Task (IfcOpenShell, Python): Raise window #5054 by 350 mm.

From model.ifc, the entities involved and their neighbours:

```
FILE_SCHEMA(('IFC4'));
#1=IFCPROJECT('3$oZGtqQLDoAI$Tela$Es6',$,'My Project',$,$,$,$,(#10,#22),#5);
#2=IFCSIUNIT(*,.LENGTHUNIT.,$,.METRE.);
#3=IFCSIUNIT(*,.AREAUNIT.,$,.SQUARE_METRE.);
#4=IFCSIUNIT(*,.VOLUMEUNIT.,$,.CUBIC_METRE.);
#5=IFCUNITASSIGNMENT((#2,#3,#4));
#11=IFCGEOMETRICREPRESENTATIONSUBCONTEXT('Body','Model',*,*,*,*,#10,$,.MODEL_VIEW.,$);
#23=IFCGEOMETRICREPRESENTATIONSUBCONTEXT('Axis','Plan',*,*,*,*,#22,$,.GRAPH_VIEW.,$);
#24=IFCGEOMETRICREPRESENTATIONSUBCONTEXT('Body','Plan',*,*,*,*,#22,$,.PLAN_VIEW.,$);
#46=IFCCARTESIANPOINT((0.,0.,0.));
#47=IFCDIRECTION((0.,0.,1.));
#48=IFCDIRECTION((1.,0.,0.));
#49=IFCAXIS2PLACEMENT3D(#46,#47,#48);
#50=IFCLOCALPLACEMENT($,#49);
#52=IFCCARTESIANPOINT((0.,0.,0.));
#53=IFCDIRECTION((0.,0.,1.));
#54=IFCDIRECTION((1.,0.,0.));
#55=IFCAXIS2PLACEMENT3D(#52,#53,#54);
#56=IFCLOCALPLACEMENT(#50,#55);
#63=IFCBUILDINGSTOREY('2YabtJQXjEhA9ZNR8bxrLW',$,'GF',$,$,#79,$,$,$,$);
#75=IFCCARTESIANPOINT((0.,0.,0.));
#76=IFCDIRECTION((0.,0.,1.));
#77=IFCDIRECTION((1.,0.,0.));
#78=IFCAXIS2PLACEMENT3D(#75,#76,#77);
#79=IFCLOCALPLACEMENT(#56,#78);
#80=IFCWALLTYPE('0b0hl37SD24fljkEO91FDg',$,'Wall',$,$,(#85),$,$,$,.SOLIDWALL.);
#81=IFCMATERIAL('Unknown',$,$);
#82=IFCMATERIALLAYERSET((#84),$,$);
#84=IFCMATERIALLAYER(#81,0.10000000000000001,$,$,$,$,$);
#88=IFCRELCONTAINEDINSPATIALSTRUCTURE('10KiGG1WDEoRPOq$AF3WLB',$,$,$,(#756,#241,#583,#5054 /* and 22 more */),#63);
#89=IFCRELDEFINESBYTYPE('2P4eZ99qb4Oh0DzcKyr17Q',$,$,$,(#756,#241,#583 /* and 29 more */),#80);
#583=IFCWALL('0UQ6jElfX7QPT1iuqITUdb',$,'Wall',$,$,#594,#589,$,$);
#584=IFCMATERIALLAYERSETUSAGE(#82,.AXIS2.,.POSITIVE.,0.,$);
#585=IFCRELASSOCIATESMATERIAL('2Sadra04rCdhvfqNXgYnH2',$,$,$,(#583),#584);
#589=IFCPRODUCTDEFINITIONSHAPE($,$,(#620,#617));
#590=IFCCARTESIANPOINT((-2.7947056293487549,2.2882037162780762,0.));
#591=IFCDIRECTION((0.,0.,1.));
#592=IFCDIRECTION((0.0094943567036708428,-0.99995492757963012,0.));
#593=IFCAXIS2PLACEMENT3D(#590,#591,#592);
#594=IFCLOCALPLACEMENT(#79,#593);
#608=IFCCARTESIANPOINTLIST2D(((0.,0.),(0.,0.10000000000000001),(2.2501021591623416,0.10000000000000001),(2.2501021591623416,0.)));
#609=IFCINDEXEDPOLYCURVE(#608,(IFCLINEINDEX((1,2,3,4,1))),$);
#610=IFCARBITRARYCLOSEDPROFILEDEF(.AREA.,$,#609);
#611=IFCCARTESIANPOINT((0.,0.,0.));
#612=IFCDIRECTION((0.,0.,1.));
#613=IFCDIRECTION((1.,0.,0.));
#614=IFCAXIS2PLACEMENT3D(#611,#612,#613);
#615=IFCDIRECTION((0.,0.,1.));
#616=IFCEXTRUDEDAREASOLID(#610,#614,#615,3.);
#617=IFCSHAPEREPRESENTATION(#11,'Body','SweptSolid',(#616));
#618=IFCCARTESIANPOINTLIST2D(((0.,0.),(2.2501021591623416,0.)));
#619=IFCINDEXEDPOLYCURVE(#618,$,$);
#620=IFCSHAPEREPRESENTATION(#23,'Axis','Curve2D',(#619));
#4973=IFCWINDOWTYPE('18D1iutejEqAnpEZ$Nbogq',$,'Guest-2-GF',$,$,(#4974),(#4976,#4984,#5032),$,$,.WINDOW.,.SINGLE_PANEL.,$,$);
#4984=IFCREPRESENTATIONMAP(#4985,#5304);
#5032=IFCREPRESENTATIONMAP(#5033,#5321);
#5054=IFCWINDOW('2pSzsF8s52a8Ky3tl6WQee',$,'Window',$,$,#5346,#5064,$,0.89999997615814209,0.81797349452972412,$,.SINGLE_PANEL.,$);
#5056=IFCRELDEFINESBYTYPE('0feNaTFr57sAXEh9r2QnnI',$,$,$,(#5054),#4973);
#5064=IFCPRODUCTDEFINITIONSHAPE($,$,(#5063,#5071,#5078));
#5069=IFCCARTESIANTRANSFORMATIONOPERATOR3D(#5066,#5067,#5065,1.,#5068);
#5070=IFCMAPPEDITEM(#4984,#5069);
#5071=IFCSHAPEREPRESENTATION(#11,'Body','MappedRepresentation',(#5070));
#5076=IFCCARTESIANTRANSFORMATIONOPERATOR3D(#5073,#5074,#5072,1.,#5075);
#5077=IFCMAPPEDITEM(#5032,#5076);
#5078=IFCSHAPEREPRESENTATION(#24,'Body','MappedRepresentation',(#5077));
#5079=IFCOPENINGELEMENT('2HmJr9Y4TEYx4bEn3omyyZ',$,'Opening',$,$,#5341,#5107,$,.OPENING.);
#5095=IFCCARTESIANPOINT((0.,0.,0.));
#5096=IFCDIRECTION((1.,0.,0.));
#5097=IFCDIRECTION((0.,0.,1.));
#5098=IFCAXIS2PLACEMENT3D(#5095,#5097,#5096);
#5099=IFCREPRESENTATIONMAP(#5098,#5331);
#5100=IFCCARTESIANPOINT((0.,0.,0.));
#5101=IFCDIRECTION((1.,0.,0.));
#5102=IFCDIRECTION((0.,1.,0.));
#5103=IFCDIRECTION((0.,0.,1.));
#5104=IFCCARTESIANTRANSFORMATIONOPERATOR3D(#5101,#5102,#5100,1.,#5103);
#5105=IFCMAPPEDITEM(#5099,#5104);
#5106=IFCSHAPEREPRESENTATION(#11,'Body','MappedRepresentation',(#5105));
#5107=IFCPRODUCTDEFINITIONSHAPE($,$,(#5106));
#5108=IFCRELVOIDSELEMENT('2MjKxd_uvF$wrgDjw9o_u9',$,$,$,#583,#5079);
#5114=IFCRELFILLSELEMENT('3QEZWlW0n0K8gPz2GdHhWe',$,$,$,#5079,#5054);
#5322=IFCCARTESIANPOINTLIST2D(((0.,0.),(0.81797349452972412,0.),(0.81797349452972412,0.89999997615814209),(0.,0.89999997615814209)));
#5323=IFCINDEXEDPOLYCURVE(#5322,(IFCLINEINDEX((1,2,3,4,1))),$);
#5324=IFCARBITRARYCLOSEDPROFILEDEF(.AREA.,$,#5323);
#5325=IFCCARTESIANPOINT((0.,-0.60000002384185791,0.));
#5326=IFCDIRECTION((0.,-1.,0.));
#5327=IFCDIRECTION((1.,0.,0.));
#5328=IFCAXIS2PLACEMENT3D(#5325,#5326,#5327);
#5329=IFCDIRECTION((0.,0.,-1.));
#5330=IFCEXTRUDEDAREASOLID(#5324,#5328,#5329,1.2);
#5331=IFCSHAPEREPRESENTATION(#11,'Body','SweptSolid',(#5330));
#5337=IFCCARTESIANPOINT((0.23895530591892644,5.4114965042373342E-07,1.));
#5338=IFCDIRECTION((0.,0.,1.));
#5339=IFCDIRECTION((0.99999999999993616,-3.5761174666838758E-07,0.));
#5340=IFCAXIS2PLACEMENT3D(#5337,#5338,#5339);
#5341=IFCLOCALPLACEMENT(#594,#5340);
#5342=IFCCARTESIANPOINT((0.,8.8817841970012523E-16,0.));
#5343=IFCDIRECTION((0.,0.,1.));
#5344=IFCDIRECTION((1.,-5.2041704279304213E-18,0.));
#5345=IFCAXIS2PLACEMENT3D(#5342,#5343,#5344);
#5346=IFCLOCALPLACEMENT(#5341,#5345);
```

```python
import numpy as np
import ifcopenshell
import ifcopenshell.api.geometry
import ifcopenshell.util.placement
import ifcopenshell.util.unit

model = ifcopenshell.open("model.ifc")
unit_scale = ifcopenshell.util.unit.calculate_unit_scale(model)

window = model.by_guid("2pSzsF8s52a8Ky3tl6WQee")
opening = window.FillsVoids[0].RelatingOpeningElement
dz = 0.35 / unit_scale

shift = np.array([0.0, 0.0, dz])
# The window is placed relative to its opening, so it follows when the opening moves.
matrix = ifcopenshell.util.placement.get_local_placement(opening.ObjectPlacement)
matrix[:3, 3] += shift
ifcopenshell.api.geometry.edit_object_placement(
    model, product=opening, matrix=matrix, is_si=False, should_transform_children=True
)

print(f"moved by {dz * unit_scale:+.3f} m")

model.write("model_updated.ifc")
```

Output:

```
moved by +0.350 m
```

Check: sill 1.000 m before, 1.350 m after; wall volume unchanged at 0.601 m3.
